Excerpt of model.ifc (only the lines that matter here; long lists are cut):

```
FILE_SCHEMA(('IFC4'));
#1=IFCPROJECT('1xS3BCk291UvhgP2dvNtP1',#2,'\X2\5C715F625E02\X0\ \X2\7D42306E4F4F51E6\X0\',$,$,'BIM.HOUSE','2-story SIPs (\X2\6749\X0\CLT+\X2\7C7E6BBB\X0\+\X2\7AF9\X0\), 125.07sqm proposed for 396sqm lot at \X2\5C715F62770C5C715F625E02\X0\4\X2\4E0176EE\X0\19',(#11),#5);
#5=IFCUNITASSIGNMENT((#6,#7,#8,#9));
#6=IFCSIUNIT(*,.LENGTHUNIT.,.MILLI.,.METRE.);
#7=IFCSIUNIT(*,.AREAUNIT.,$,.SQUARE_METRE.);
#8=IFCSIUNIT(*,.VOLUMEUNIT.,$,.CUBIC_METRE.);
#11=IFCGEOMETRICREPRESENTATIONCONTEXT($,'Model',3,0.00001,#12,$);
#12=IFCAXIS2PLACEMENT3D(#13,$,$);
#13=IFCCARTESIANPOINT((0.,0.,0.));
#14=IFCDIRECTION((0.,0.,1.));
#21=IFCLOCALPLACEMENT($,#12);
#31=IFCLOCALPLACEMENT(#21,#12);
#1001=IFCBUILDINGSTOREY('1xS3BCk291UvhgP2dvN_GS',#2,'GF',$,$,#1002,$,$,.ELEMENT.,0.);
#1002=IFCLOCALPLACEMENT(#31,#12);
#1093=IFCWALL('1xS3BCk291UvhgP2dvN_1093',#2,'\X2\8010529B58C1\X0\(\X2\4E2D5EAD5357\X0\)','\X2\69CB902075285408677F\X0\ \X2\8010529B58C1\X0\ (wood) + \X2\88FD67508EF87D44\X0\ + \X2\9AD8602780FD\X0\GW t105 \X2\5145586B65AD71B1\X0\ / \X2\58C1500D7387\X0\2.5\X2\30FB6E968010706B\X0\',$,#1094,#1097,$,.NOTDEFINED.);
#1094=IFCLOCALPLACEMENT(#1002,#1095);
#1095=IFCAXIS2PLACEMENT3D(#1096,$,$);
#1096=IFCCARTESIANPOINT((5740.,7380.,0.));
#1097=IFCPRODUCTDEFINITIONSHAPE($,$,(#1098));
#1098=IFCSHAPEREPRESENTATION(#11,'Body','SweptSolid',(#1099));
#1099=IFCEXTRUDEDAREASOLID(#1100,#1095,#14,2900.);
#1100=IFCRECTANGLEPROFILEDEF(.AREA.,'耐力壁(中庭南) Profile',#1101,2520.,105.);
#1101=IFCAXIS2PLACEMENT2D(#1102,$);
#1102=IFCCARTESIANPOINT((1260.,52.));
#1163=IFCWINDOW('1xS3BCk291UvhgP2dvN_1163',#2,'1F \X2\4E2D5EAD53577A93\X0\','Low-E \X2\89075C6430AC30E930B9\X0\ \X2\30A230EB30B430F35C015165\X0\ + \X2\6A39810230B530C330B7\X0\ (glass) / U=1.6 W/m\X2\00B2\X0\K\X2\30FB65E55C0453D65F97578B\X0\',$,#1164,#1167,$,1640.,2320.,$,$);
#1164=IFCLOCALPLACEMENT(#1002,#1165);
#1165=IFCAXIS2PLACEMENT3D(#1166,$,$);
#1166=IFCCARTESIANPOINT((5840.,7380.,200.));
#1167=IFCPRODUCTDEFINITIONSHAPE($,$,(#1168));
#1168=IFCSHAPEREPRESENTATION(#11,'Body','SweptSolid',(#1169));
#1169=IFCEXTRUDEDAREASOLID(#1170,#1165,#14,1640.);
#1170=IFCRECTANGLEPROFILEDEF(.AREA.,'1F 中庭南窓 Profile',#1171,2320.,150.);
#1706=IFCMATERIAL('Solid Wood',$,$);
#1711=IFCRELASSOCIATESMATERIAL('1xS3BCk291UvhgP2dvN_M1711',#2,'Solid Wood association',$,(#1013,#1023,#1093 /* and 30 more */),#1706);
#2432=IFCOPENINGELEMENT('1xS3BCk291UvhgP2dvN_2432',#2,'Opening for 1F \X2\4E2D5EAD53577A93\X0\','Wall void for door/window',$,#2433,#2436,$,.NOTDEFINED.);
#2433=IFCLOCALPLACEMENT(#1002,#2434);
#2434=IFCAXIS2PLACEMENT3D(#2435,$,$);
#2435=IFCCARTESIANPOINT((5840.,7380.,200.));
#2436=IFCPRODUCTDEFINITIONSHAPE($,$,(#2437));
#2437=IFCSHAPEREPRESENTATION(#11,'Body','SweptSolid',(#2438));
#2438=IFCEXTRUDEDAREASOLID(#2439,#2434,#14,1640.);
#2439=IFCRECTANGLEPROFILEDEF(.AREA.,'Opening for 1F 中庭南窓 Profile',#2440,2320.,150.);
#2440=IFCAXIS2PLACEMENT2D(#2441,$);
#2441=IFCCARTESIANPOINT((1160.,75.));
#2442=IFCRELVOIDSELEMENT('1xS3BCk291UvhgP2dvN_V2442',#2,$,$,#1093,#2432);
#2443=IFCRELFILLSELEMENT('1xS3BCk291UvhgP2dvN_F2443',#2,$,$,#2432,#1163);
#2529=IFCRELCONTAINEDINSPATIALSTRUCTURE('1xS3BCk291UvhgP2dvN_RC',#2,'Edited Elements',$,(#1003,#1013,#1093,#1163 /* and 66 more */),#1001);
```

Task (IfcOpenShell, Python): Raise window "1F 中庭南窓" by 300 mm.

```python
import numpy as np
import ifcopenshell
import ifcopenshell.api.geometry
import ifcopenshell.util.placement
import ifcopenshell.util.unit

model = ifcopenshell.open("model.ifc")
unit_scale = ifcopenshell.util.unit.calculate_unit_scale(model)

window = model.by_guid("1xS3BCk291UvhgP2dvN_1163")
opening = window.FillsVoids[0].RelatingOpeningElement
dz = 0.3 / unit_scale

shift = np.array([0.0, 0.0, dz])
# The window is not placed relative to its opening, so move both.
for product in (opening, window):
    matrix = ifcopenshell.util.placement.get_local_placement(product.ObjectPlacement)
    matrix[:3, 3] += shift
    ifcopenshell.api.geometry.edit_object_placement(model, product=product, matrix=matrix, is_si=False)

print(f"moved by {dz * unit_scale:+.3f} m")

model.write("model_edited.ifc")
```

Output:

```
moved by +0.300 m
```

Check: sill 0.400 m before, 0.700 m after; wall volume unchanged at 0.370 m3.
